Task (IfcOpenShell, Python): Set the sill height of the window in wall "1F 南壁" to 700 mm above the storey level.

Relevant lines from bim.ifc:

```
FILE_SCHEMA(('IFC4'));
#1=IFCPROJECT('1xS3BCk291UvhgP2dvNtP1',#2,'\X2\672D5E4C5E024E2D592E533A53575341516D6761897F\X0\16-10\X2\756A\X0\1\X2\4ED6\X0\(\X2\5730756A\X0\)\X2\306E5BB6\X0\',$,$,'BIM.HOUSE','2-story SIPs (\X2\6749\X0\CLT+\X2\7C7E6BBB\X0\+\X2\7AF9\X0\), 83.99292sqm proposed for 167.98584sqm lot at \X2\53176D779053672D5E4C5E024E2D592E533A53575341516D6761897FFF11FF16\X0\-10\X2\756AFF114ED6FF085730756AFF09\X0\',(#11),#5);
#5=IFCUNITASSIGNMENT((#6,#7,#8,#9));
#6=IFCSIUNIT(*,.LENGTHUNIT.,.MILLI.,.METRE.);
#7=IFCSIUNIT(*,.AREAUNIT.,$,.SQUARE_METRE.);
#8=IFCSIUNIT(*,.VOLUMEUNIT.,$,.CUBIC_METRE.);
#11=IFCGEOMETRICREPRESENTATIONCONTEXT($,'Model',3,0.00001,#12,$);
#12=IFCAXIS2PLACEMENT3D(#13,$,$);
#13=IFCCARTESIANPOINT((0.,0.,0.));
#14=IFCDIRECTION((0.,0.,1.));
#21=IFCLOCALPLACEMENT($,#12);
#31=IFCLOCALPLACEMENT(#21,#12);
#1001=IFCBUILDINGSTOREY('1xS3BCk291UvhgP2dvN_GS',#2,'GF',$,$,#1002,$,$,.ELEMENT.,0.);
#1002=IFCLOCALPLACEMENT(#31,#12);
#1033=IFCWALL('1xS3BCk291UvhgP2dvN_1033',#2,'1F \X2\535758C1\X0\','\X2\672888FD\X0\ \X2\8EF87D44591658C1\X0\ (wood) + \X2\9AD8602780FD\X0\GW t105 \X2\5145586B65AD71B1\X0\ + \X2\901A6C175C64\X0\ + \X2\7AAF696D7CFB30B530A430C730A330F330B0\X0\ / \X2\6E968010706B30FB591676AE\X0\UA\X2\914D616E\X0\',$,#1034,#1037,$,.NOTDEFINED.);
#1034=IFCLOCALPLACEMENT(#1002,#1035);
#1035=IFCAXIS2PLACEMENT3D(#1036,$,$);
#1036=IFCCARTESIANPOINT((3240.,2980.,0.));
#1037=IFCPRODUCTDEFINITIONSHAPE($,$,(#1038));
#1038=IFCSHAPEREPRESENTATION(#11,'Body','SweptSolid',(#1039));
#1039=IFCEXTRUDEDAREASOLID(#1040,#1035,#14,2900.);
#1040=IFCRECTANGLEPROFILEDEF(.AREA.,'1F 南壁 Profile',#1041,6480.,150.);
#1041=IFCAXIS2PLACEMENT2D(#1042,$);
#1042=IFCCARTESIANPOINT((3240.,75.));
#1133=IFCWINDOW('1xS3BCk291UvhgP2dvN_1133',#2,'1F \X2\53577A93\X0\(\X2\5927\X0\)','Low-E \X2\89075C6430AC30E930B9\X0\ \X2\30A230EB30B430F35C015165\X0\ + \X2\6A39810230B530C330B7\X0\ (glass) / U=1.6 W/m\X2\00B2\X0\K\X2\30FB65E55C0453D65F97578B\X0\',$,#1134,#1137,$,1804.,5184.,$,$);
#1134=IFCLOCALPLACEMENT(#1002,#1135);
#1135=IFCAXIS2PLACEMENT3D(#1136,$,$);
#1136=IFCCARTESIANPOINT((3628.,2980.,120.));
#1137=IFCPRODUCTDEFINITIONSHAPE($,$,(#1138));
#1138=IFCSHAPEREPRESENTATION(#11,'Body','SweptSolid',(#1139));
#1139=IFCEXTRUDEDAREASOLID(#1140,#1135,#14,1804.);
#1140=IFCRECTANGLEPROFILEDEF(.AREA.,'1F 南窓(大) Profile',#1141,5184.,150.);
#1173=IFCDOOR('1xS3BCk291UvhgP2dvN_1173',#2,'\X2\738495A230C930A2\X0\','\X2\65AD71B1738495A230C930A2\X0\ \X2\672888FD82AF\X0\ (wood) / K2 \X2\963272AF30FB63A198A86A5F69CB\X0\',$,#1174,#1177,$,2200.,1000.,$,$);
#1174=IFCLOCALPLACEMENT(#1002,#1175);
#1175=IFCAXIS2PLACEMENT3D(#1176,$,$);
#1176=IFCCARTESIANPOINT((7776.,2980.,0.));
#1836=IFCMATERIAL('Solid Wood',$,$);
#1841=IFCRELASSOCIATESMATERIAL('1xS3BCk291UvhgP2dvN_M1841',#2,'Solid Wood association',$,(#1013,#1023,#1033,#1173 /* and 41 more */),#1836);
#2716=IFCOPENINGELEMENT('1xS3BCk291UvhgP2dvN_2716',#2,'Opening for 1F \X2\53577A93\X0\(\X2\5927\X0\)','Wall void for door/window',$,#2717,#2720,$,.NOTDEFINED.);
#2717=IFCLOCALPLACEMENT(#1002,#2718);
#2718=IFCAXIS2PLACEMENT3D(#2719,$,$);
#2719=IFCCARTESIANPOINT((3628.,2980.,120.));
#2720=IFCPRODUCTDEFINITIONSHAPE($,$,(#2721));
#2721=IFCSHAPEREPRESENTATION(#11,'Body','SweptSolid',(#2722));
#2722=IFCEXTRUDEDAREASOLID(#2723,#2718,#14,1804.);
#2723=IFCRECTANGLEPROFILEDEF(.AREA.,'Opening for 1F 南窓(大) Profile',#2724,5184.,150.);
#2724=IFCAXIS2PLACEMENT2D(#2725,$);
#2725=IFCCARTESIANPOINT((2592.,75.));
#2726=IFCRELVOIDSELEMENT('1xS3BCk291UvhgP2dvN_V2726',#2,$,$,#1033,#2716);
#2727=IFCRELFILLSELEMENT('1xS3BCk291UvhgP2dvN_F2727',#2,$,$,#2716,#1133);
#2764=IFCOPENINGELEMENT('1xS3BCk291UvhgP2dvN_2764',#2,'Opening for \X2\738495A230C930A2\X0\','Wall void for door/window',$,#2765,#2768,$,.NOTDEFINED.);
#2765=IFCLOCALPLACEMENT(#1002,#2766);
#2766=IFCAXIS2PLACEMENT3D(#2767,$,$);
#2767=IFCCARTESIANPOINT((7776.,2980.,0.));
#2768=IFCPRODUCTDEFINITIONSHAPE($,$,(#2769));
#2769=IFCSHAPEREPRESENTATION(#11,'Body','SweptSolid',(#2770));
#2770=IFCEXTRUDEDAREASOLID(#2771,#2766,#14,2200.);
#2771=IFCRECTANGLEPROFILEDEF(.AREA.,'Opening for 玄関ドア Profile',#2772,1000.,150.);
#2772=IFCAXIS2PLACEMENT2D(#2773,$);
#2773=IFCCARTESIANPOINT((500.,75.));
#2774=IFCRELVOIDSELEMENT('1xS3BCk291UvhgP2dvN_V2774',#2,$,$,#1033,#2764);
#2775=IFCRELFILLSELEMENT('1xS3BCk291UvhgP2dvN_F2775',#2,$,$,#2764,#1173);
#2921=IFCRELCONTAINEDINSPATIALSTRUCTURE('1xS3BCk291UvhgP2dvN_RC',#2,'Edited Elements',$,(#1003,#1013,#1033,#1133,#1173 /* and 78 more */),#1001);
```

```python
import numpy as np
import ifcopenshell
import ifcopenshell.api.geometry
import ifcopenshell.geom
import ifcopenshell.util.element
import ifcopenshell.util.placement
import ifcopenshell.util.shape
import ifcopenshell.util.unit

model = ifcopenshell.open("bim.ifc")
unit_scale = ifcopenshell.util.unit.calculate_unit_scale(model)

window = model.by_id(1133)
opening = window.FillsVoids[0].RelatingOpeningElement
storey = ifcopenshell.util.element.get_container(window, ifc_class="IfcBuildingStorey")
level = ifcopenshell.util.placement.get_local_placement(storey.ObjectPlacement)[2, 3]

# The opening's origin need not be at the sill, so measure its lowest point.
shape = ifcopenshell.geom.create_shape(ifcopenshell.geom.settings(), opening)
bottom = ifcopenshell.util.shape.get_shape_bottom_elevation(shape, shape.geometry) / unit_scale
dz = level + 700.0 - bottom

shift = np.array([0.0, 0.0, dz])
# The window is not placed relative to its opening, so move both.
for product in (opening, window):
    matrix = ifcopenshell.util.placement.get_local_placement(product.ObjectPlacement)
    matrix[:3, 3] += shift
    ifcopenshell.api.geometry.edit_object_placement(model, product=product, matrix=matrix, is_si=False)

print(f"moved by {dz * unit_scale:+.3f} m")

model.write("bim_updated.ifc")
```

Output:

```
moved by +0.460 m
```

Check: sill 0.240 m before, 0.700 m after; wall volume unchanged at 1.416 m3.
